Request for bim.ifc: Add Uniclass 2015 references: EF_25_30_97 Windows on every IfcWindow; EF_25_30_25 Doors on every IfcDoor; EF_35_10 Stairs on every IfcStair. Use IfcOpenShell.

First a look at what the model holds.

```python
import ifcopenshell

model = ifcopenshell.open("bim.ifc")
print(model.schema)
print("classifications:", [c.Name for c in model.by_type("IfcClassification")])
for ifc_class in ("IfcDoor", "IfcRoof", "IfcStair", "IfcWall", "IfcWindow"):
    print(ifc_class, len(model.by_type(ifc_class)))
```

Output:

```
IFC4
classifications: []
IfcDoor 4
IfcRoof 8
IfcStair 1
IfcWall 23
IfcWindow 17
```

```python
import ifcopenshell
import ifcopenshell.api.classification

model = ifcopenshell.open("bim.ifc")

system = ifcopenshell.api.classification.add_classification(model, classification="Uniclass 2015")

codes = {
    "IfcWindow": ("EF_25_30_97", "Windows"),
    "IfcDoor": ("EF_25_30_25", "Doors"),
    "IfcStair": ("EF_35_10", "Stairs"),
}
for ifc_class, (code, name) in codes.items():
    products = model.by_type(ifc_class)
    ifcopenshell.api.classification.add_reference(
        model, products=products, classification=system, identification=code, name=name
    )
    print(code, len(products))

model.write("bim-out.ifc")
```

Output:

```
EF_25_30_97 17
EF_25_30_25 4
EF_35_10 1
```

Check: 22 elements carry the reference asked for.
